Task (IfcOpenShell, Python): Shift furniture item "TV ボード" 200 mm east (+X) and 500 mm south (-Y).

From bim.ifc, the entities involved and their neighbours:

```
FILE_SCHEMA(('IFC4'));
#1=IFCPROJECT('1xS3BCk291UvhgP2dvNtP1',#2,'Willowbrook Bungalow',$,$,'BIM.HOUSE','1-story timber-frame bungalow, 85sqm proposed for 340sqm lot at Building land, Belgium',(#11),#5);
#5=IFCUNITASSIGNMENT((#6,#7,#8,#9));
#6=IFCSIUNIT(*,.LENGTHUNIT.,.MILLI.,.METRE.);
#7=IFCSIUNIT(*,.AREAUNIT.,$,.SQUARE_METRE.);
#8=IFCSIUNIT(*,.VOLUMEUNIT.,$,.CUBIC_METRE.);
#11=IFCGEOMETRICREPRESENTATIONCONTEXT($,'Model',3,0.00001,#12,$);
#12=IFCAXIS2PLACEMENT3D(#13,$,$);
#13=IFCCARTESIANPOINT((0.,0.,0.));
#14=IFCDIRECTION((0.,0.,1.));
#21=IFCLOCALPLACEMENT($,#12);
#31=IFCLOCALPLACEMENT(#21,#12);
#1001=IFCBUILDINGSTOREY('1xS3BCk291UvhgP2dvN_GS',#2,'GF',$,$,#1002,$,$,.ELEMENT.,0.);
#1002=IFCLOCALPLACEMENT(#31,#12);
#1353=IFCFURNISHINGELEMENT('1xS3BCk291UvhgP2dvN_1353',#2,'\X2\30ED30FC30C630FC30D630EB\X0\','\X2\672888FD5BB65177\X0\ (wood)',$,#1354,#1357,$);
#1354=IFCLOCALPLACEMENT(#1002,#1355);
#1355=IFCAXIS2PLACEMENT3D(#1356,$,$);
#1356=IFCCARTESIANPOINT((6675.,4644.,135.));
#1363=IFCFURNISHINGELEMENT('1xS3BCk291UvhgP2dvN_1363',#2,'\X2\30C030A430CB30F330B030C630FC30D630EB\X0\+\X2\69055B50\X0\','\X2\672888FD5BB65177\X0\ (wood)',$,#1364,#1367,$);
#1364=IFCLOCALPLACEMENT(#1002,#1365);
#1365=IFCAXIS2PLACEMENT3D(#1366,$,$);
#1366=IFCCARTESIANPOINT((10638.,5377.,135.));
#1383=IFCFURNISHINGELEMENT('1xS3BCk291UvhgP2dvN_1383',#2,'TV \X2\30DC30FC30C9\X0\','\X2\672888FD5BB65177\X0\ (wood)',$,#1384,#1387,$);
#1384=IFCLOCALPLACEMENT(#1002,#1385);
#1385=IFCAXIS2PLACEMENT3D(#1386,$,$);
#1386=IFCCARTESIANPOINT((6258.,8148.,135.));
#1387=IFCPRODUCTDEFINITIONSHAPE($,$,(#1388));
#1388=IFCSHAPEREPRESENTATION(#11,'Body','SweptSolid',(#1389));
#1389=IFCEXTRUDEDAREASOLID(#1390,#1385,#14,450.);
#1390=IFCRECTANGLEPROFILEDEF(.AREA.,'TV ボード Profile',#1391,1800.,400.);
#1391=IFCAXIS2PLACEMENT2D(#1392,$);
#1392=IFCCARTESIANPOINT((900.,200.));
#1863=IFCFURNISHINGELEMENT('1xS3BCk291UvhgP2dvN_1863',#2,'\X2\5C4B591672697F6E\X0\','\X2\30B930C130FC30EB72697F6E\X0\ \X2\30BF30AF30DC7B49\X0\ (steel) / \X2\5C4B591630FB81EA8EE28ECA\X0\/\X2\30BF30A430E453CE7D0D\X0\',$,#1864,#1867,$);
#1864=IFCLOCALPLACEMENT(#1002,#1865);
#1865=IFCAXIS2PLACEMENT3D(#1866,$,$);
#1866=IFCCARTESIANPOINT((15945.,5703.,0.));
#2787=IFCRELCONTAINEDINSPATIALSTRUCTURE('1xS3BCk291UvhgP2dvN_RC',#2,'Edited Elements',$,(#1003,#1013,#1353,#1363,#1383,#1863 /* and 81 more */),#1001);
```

```python
import ifcopenshell
import ifcopenshell.api.geometry
import ifcopenshell.util.placement
import ifcopenshell.util.unit

model = ifcopenshell.open("bim.ifc")
unit_scale = ifcopenshell.util.unit.calculate_unit_scale(model)

item = model.by_guid("1xS3BCk291UvhgP2dvN_1383")
matrix = ifcopenshell.util.placement.get_local_placement(item.ObjectPlacement)
matrix[0, 3] += 0.2 / unit_scale
matrix[1, 3] -= 0.5 / unit_scale
ifcopenshell.api.geometry.edit_object_placement(model, product=item, matrix=matrix, is_si=False)

print(ifcopenshell.util.placement.get_local_placement(item.ObjectPlacement).round(3) + 0.0)

model.write("bim_v2.ifc")
```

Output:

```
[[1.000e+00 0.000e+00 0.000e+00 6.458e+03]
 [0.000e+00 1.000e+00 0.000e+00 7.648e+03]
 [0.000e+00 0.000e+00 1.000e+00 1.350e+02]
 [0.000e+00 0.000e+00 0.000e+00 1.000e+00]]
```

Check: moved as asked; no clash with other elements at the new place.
